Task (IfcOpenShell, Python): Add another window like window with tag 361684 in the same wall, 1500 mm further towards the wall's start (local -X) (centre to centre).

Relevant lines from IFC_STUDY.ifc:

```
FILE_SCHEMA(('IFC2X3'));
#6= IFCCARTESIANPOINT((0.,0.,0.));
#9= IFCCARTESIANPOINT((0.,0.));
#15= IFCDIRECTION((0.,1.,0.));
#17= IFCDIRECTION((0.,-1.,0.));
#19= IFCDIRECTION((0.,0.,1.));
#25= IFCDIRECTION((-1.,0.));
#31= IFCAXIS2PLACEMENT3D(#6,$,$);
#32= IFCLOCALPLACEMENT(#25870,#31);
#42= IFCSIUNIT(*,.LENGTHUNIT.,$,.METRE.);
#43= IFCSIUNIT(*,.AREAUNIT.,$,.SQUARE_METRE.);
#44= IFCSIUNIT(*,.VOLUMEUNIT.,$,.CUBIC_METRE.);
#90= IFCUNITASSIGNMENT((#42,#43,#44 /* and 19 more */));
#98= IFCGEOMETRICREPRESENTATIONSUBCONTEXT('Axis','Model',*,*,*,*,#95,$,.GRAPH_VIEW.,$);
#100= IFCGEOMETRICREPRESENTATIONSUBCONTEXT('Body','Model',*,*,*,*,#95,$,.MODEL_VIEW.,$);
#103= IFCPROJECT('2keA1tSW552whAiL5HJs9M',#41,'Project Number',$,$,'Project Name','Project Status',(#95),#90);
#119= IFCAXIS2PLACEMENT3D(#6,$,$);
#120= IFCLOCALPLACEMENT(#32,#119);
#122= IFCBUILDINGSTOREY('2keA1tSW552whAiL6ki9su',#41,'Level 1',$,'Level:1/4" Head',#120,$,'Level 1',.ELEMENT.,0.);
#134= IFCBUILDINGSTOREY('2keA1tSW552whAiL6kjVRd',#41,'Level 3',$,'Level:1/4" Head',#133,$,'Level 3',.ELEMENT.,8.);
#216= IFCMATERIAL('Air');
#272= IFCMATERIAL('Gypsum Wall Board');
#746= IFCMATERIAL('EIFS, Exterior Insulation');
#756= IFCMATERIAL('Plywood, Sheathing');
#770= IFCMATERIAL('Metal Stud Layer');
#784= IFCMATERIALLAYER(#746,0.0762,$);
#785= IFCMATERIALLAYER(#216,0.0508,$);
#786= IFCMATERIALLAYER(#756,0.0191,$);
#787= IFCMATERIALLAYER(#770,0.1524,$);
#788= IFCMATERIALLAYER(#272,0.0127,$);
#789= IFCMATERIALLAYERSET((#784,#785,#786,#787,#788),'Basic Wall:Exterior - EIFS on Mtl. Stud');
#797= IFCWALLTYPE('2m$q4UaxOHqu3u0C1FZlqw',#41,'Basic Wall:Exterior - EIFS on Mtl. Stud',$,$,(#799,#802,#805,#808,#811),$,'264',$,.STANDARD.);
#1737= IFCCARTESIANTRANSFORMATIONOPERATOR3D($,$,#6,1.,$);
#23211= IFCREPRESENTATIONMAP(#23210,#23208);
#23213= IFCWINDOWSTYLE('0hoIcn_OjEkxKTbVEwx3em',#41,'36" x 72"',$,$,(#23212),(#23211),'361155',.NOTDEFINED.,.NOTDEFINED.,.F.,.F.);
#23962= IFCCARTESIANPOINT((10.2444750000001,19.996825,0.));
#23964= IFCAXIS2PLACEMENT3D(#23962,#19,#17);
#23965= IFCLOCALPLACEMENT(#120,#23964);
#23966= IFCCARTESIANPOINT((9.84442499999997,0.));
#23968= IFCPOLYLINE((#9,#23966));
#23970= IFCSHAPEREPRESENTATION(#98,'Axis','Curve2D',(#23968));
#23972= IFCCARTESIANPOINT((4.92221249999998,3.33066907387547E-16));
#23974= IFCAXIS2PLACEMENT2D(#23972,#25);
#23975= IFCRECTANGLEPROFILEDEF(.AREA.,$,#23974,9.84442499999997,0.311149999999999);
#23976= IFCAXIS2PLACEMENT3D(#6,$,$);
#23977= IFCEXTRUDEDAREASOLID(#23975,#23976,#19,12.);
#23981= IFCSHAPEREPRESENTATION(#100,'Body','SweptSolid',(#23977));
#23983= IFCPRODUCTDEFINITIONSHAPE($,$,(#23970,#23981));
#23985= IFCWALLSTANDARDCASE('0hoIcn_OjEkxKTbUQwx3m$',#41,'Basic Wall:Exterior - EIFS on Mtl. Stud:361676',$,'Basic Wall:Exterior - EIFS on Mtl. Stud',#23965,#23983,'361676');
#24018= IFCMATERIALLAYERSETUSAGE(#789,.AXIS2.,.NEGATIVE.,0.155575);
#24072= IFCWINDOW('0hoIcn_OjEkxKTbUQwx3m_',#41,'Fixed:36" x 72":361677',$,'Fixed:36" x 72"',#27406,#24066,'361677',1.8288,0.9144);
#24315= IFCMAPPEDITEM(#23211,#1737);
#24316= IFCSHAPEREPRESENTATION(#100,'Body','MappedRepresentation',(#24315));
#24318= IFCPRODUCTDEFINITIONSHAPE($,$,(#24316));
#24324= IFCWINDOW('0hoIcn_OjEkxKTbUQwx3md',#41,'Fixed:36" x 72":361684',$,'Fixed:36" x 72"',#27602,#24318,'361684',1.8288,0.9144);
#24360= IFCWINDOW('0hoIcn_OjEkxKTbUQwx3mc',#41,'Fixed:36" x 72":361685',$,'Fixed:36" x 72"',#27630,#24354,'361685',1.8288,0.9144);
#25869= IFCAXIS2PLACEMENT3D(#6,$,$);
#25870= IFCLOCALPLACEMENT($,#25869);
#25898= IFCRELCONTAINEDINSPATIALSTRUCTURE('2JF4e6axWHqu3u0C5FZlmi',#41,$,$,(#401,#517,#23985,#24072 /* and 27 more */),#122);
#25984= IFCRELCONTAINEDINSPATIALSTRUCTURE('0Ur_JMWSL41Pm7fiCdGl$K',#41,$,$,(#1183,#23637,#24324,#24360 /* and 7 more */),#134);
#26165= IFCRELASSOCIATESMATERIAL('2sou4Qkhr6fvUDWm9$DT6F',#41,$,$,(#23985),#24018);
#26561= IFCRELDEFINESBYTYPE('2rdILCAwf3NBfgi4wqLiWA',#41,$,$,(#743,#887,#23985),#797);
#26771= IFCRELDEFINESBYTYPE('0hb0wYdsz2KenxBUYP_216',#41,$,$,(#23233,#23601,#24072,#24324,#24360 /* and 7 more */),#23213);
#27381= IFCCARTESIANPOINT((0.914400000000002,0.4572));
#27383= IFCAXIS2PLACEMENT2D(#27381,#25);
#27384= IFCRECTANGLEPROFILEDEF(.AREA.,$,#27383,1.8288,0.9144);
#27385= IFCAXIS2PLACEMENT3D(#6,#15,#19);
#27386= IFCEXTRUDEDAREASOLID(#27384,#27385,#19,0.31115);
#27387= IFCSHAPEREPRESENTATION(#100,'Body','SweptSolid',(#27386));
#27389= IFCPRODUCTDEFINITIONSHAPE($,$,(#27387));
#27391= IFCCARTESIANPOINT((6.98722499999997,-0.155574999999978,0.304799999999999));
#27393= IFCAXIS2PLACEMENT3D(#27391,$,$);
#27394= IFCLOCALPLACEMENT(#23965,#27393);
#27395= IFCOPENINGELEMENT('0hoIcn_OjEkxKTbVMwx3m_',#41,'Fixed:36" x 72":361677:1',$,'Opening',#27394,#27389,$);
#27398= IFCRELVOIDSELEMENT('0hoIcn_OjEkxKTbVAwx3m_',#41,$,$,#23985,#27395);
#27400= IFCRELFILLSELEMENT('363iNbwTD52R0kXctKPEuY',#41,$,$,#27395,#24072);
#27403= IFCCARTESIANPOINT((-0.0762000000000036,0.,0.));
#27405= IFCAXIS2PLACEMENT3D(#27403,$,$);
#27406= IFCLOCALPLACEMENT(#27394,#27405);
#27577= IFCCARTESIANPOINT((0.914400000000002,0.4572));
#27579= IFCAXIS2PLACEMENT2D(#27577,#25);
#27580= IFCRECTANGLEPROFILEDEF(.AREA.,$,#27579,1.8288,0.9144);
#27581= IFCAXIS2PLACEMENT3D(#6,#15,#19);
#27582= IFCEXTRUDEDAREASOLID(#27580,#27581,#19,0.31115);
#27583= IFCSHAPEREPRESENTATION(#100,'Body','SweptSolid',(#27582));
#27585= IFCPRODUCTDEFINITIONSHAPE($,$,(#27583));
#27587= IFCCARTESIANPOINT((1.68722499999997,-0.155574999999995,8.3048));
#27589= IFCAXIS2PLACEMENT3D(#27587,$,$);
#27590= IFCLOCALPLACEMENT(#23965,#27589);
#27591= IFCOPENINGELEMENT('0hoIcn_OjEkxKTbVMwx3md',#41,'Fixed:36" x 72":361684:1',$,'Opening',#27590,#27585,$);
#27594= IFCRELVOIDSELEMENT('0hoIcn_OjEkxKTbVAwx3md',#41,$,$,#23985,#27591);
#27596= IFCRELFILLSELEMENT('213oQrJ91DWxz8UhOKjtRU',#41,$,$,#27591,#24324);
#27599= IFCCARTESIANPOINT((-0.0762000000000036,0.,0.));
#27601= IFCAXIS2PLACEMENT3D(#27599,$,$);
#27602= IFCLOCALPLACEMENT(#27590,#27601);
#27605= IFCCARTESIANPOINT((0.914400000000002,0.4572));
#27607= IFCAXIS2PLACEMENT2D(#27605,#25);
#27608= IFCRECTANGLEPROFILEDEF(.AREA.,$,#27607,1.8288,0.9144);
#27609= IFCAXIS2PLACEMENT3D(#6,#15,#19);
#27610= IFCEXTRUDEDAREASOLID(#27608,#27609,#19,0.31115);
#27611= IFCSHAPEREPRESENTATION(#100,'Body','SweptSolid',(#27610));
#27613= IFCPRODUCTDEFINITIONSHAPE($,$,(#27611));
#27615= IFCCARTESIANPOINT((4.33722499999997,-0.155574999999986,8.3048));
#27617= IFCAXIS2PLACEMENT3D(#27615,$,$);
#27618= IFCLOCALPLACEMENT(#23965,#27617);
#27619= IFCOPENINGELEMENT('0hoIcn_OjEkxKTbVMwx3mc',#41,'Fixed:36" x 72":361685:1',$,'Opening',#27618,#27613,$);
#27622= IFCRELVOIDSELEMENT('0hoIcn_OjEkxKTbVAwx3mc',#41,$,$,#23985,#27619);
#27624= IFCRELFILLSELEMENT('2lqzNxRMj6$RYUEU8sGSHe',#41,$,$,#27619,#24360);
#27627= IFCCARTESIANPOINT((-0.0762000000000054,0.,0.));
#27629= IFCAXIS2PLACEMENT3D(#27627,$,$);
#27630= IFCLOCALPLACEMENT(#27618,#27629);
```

```python
import ifcopenshell
import ifcopenshell.api.feature
import ifcopenshell.api.geometry
import ifcopenshell.api.root
import ifcopenshell.geom
import ifcopenshell.util.element
import ifcopenshell.util.placement
import ifcopenshell.util.shape
import ifcopenshell.util.unit

model = ifcopenshell.open("IFC_STUDY.ifc")
unit_scale = ifcopenshell.util.unit.calculate_unit_scale(model)
settings = ifcopenshell.geom.settings()


def volume(element):
    """Net volume in cubic metres, openings subtracted."""
    shape = ifcopenshell.geom.create_shape(settings, element)
    return ifcopenshell.util.shape.get_volume(shape.geometry)


def reuse_history(source, copy):
    """copy_class also copies each property set's owner history, people and application; keep the originals."""
    for rel in copy.IsDefinedBy:
        if rel.is_a("IfcRelDefinesByProperties") and (history := rel.RelatingPropertyDefinition.OwnerHistory):
            rel.RelatingPropertyDefinition.OwnerHistory = source.OwnerHistory
            ifcopenshell.util.element.remove_deep2(model, history)


window = model.by_guid("0hoIcn_OjEkxKTbUQwx3md")
opening = window.FillsVoids[0].RelatingOpeningElement
wall = opening.VoidsElements[0].RelatingBuildingElement
before = volume(wall)
shift = ifcopenshell.util.placement.get_local_placement(wall.ObjectPlacement)[:3, 0] * -1.5 / unit_scale

# copy_class copies the void relationship, type, container and properties, but no geometry.
new_opening = ifcopenshell.api.root.copy_class(model, product=opening)
new_opening.Representation = ifcopenshell.util.element.copy_deep(
    model, opening.Representation, exclude=["IfcGeometricRepresentationContext", "IfcRepresentationMap"]
)
new_opening.Name = 'Fixed:36" x 72"'
new_window = ifcopenshell.api.root.copy_class(model, product=window)
new_window.Representation = ifcopenshell.util.element.copy_deep(
    model, window.Representation, exclude=["IfcGeometricRepresentationContext", "IfcRepresentationMap"]
)
new_window.Name = 'Fixed:36" x 72"'
new_window.Tag = None
reuse_history(window, new_window)
fills = ifcopenshell.api.feature.add_filling(model, opening=new_opening, element=new_window)
fills.OwnerHistory = new_window.OwnerHistory  # required in IFC2X3

for old, new in ((opening, new_opening), (window, new_window)):
    matrix = ifcopenshell.util.placement.get_local_placement(old.ObjectPlacement)
    matrix[:3, 3] += shift
    ifcopenshell.api.geometry.edit_object_placement(model, product=new, matrix=matrix, is_si=False)

after = volume(wall)

print(f"wall volume {before:.3f} -> {after:.3f} m3")

model.write("IFC_STUDY-out.ifc")
```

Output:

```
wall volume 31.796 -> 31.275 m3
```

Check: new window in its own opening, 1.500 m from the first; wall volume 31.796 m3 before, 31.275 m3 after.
